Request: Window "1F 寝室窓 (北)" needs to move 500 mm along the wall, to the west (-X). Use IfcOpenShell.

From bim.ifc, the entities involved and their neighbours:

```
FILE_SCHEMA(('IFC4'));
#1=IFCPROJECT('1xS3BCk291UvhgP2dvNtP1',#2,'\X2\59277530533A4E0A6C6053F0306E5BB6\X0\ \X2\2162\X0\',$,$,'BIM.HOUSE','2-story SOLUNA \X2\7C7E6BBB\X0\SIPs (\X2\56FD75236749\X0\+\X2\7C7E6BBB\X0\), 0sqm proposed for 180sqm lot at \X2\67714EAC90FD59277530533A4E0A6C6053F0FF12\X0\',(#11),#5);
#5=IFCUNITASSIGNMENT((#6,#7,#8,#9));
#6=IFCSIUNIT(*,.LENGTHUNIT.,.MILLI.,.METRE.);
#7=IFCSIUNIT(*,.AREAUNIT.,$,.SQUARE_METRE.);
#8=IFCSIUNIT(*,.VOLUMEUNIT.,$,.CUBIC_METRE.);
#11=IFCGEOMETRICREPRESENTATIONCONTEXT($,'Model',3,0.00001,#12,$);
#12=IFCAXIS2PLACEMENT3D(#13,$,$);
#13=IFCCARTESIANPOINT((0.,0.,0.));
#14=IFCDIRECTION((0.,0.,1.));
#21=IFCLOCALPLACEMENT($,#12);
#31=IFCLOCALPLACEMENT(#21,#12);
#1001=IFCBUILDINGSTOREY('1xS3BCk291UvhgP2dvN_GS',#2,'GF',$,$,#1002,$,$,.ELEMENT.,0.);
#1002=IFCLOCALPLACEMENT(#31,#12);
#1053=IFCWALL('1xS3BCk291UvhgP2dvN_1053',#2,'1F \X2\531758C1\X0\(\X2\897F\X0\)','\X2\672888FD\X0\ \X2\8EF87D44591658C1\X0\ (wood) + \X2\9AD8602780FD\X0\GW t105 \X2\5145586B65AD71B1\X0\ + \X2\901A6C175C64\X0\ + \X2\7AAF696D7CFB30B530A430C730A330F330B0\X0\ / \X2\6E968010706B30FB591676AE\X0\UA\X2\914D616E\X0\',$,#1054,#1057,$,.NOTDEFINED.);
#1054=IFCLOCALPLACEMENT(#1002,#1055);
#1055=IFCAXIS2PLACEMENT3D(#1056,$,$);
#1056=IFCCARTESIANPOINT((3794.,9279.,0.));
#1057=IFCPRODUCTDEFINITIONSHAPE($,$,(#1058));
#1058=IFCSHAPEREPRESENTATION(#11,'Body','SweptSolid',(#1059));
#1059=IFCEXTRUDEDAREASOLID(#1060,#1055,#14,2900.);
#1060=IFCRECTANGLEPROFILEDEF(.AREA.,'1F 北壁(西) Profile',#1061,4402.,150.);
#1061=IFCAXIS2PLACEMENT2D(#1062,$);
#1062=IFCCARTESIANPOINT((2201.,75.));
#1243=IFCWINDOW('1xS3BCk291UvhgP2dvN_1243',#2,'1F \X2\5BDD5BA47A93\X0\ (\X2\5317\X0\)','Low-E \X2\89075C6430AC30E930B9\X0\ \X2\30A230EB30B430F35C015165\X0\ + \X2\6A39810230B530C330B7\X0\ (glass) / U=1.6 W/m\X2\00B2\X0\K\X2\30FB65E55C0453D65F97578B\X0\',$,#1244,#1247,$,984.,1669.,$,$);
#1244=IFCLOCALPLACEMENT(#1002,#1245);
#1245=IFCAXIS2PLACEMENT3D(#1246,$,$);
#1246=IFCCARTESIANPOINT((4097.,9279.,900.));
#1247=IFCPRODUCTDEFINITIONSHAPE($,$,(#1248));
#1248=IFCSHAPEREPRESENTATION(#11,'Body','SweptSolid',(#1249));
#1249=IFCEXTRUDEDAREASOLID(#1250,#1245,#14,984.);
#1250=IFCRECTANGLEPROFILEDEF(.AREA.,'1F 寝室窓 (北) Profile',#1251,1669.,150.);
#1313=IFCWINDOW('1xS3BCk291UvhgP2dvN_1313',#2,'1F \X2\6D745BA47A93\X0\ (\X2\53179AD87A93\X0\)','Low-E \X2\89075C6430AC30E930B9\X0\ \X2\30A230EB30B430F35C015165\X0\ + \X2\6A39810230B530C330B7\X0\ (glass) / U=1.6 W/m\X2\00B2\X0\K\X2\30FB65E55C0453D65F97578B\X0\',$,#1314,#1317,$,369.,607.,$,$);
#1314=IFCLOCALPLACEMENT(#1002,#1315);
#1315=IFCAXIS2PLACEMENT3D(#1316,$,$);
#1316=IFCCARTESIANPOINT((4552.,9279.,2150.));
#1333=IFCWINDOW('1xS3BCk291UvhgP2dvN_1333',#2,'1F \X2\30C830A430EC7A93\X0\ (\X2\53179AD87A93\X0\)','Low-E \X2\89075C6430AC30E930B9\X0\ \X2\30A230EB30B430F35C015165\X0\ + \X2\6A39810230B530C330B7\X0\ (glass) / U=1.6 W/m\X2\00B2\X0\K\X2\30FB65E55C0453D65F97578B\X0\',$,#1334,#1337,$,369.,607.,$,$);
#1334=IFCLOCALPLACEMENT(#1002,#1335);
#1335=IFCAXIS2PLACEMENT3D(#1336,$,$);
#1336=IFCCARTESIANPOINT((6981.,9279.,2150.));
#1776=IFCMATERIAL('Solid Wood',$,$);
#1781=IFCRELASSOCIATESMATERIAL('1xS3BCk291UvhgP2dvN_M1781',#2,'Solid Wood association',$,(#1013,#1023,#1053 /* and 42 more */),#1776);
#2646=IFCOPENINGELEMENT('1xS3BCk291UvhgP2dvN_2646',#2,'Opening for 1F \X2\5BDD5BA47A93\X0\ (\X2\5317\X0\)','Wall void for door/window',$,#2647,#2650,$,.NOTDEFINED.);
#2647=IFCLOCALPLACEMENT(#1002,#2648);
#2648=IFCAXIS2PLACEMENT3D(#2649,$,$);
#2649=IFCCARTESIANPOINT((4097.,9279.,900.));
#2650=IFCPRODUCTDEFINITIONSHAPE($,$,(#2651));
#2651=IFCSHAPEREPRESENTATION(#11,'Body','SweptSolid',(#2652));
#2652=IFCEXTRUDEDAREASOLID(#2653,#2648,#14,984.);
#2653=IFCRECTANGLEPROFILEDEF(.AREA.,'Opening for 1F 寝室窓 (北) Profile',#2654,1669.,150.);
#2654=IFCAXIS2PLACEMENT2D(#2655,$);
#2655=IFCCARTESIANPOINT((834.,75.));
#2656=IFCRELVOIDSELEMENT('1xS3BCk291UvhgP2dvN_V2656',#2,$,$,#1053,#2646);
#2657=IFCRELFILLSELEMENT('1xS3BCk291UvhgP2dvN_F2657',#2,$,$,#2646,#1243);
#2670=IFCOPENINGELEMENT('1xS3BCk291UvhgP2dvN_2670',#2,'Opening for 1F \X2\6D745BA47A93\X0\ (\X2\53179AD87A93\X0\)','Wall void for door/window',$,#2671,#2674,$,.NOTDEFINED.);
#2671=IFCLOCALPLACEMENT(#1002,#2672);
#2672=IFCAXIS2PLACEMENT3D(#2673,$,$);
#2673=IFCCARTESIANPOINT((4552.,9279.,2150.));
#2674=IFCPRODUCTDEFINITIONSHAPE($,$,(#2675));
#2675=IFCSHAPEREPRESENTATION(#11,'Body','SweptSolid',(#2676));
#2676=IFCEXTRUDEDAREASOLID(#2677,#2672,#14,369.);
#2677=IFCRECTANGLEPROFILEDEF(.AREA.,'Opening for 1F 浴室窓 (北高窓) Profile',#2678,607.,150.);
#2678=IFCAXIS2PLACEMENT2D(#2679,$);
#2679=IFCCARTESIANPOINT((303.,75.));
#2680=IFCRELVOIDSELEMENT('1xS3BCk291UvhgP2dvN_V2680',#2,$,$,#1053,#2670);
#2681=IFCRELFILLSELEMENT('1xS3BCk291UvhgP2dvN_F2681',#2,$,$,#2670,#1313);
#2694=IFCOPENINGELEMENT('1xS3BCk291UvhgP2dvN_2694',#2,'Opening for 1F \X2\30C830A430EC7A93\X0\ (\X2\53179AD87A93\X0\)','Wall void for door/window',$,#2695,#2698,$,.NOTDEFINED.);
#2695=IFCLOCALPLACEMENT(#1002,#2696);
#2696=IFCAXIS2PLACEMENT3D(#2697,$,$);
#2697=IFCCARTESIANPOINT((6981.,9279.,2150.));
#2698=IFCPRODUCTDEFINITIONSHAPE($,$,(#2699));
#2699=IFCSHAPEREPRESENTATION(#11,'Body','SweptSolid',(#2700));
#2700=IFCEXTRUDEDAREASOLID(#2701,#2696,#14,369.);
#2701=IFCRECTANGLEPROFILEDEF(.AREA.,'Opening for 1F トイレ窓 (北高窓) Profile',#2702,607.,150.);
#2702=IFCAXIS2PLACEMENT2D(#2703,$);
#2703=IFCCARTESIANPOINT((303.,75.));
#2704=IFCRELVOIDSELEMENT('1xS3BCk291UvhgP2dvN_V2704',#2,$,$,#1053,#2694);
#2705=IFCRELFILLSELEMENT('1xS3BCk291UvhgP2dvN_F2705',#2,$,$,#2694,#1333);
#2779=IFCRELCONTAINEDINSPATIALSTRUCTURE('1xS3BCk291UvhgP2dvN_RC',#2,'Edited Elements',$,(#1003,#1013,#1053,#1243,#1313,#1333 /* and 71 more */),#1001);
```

```python
import ifcopenshell
import ifcopenshell.api.geometry
import ifcopenshell.util.placement

model = ifcopenshell.open("bim.ifc")

window = model.by_guid("1xS3BCk291UvhgP2dvN_1243")
opening = window.FillsVoids[0].RelatingOpeningElement
wall = opening.VoidsElements[0].RelatingBuildingElement

wall_matrix = ifcopenshell.util.placement.get_local_placement(wall.ObjectPlacement)
shift = wall_matrix[:3, 0] * -500.0
before = ifcopenshell.util.placement.get_local_placement(window.ObjectPlacement)[:3, 3].copy()

# The window is not placed relative to its opening, so move both.
for product in (opening, window):
    matrix = ifcopenshell.util.placement.get_local_placement(product.ObjectPlacement)
    matrix[:3, 3] += shift
    ifcopenshell.api.geometry.edit_object_placement(model, product=product, matrix=matrix, is_si=False)

after = ifcopenshell.util.placement.get_local_placement(window.ObjectPlacement)[:3, 3]
print("window moved by", (after - before).round(3) + 0.0)

model.write("bim_rev.ifc")
```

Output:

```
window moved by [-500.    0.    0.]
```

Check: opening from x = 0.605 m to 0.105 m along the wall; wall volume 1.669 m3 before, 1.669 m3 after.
